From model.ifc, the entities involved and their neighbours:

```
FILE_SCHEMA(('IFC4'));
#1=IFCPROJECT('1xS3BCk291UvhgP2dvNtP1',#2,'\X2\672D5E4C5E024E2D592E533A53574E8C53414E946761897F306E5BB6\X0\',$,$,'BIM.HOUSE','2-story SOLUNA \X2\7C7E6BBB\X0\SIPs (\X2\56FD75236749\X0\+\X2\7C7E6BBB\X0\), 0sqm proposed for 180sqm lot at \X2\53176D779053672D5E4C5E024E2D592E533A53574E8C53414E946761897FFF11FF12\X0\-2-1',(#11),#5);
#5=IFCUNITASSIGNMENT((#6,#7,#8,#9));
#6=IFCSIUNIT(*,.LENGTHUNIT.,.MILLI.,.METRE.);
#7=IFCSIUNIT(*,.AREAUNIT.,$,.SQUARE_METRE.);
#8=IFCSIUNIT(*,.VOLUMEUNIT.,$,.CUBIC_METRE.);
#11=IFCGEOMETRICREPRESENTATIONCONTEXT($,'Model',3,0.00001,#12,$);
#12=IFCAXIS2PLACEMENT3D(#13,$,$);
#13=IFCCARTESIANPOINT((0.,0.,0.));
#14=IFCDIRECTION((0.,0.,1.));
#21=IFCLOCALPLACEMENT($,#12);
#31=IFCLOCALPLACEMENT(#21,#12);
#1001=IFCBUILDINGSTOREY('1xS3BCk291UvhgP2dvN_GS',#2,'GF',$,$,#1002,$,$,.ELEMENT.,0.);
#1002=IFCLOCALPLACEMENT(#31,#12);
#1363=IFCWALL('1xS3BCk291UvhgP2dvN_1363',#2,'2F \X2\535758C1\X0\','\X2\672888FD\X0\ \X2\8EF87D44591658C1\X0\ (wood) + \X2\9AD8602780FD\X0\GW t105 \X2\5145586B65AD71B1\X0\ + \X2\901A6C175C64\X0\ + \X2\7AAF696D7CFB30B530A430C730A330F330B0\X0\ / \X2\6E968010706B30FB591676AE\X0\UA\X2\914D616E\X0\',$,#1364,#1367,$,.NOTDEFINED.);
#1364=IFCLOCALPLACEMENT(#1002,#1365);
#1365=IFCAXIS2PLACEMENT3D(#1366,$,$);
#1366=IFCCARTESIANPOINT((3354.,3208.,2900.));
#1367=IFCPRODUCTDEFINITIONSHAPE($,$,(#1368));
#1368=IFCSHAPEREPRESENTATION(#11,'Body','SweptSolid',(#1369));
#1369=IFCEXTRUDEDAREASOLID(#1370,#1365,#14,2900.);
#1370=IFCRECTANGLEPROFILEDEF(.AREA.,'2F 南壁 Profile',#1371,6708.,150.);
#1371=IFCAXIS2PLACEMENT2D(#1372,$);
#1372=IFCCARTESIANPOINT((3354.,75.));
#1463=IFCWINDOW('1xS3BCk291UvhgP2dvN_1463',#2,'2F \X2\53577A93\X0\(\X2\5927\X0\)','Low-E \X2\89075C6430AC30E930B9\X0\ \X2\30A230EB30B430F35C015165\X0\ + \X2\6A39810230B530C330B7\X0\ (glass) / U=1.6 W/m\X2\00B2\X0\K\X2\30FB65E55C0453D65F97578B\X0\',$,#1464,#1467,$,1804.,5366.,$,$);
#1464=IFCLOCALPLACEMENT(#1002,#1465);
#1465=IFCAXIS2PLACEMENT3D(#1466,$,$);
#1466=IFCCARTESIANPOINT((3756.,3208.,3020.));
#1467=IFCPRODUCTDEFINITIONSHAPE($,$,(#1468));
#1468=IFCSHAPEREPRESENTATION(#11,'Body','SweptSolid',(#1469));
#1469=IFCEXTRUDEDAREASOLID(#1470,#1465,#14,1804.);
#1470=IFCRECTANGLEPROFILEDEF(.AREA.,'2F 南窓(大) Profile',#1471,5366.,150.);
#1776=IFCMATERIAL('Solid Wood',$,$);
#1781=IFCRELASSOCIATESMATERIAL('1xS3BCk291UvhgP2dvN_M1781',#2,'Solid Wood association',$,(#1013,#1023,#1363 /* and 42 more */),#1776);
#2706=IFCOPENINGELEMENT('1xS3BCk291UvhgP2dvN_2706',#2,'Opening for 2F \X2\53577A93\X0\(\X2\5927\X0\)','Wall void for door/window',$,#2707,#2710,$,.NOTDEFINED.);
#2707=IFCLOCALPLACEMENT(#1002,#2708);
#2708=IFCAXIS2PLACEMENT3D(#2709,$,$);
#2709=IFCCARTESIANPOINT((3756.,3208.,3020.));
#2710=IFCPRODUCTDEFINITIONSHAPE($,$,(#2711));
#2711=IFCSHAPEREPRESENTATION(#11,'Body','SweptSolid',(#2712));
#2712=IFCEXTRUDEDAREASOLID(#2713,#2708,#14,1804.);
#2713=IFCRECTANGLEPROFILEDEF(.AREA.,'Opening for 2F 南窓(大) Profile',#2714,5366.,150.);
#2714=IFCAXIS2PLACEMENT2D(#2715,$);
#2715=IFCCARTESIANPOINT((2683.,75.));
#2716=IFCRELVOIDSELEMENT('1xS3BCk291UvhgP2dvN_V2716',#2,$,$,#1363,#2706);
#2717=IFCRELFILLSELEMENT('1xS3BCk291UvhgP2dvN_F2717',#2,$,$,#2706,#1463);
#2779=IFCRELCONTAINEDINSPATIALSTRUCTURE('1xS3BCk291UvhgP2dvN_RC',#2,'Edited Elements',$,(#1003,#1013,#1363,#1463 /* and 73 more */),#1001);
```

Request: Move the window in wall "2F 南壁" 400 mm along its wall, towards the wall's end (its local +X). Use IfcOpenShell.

```python
import ifcopenshell
import ifcopenshell.api.geometry
import ifcopenshell.util.placement
import ifcopenshell.util.unit

model = ifcopenshell.open("model.ifc")
unit_scale = ifcopenshell.util.unit.calculate_unit_scale(model)

window = model.by_guid("1xS3BCk291UvhgP2dvN_1463")
opening = window.FillsVoids[0].RelatingOpeningElement
wall = opening.VoidsElements[0].RelatingBuildingElement

wall_matrix = ifcopenshell.util.placement.get_local_placement(wall.ObjectPlacement)
shift = wall_matrix[:3, 0] * 0.4 / unit_scale
before = ifcopenshell.util.placement.get_local_placement(window.ObjectPlacement)[:3, 3].copy()

# The window is not placed relative to its opening, so move both.
for product in (opening, window):
    matrix = ifcopenshell.util.placement.get_local_placement(product.ObjectPlacement)
    matrix[:3, 3] += shift
    ifcopenshell.api.geometry.edit_object_placement(model, product=product, matrix=matrix, is_si=False)

after = ifcopenshell.util.placement.get_local_placement(window.ObjectPlacement)[:3, 3]
print("window moved by", (after - before).round(3) + 0.0)

model.write("model_updated.ifc")
```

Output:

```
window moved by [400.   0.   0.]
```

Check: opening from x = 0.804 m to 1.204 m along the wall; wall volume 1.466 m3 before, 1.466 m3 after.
